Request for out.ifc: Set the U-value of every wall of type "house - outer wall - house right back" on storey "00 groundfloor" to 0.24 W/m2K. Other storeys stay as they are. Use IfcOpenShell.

First a look at what the model holds.

```python
import ifcopenshell
import ifcopenshell.util.element

model = ifcopenshell.open("out.ifc")
print(model.schema)
storey = next(s for s in model.by_type("IfcBuildingStorey") if s.Name == "00 groundfloor")
walls = [e for e in ifcopenshell.util.element.get_decomposition(storey) if e.is_a("IfcWall")]
seen = {}
for e in walls:
    element_type = ifcopenshell.util.element.get_type(e)
    key = (element_type.Name if element_type != e and element_type else None, ifcopenshell.util.element.get_pset(e, "Pset_WallCommon", "ThermalTransmittance"))
    seen[key] = seen.get(key, 0) + 1
for (name, value), count in sorted(seen.items(), key=str):
    print(count, "x", name, "|", value)
```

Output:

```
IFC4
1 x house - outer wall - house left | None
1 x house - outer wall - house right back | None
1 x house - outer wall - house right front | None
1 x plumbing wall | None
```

```python
import ifcopenshell
import ifcopenshell.api.pset
import ifcopenshell.util.element

model = ifcopenshell.open("out.ifc")

storey = next(s for s in model.by_type("IfcBuildingStorey") if s.Name == "00 groundfloor")
walls = [e for e in ifcopenshell.util.element.get_decomposition(storey) if e.is_a("IfcWall")]

count = 0
for e in walls:
    element_type = ifcopenshell.util.element.get_type(e)
    if element_type in (None, e) or element_type.Name != "house - outer wall - house right back":
        continue
    # add_pset returns the element's existing set when there is one.
    pset = ifcopenshell.api.pset.add_pset(model, product=e, name="Pset_WallCommon")
    ifcopenshell.api.pset.edit_pset(model, pset=pset, properties={"ThermalTransmittance": 0.24})
    count += 1

print(count, "walls updated")

model.write("out_rev.ifc")
```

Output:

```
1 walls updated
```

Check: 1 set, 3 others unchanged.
